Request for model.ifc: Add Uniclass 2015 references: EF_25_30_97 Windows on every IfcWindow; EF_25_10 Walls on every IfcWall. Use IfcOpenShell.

First a look at what the model holds.

```python
import ifcopenshell

model = ifcopenshell.open("model.ifc")
print(model.schema)
print("classifications:", [c.Name for c in model.by_type("IfcClassification")])
for ifc_class in ("IfcDoor", "IfcRoof", "IfcStair", "IfcWall", "IfcWindow"):
    print(ifc_class, len(model.by_type(ifc_class)))
```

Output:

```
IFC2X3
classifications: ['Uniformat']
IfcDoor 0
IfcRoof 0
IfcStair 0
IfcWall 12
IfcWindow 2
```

```python
import ifcopenshell
import ifcopenshell.api.classification

model = ifcopenshell.open("model.ifc")

# IFC2X3 requires Source and Edition and has no link from the project to the system.
system = model.create_entity("IfcClassification", Source="NBS", Edition="2015", Name="Uniclass 2015")

codes = {
    "IfcWindow": ("EF_25_30_97", "Windows"),
    "IfcWall": ("EF_25_10", "Walls"),
}
for ifc_class, (code, name) in codes.items():
    products = model.by_type(ifc_class)
    ifcopenshell.api.classification.add_reference(
        model, products=products, classification=system, identification=code, name=name
    )
    print(code, len(products))

model.write("model_edited.ifc")
```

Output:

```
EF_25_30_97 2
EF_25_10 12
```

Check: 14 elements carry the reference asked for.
